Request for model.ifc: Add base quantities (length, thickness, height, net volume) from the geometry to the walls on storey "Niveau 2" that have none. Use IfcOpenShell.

First a look at what the model holds.

```python
import ifcopenshell
import ifcopenshell.util.element
import ifcopenshell.util.unit

model = ifcopenshell.open("model.ifc")
print(model.schema)
for unit_type in ("LENGTHUNIT", "AREAUNIT", "VOLUMEUNIT"):
    print(unit_type, ifcopenshell.util.unit.calculate_unit_scale(model, unit_type))
storey = next(s for s in model.by_type("IfcBuildingStorey") if s.Name == "Niveau 2")
walls = [e for e in ifcopenshell.util.element.get_decomposition(storey) if e.is_a("IfcWall")]
for e in sorted(walls, key=lambda e: e.id()):
    print(e.id(), e.is_a(), e.Name, list(ifcopenshell.util.element.get_psets(e, qtos_only=True)), sep=" | ")
```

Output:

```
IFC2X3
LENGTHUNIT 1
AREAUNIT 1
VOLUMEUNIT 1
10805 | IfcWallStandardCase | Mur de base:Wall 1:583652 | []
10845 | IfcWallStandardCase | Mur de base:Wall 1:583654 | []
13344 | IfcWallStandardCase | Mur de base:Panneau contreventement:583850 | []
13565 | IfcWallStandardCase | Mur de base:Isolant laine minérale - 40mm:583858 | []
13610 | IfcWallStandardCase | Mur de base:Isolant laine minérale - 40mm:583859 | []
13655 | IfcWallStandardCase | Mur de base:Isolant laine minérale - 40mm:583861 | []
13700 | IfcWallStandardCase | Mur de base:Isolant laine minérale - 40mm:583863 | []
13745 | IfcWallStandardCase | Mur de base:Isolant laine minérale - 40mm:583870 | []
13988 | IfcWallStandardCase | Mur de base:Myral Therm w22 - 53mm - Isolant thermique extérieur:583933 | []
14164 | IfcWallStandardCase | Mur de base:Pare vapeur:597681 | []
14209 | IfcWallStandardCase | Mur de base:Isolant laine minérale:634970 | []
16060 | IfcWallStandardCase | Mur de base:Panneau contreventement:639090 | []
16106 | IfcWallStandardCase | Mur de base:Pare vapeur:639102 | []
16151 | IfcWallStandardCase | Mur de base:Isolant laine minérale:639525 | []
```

```python
import ifcopenshell
import ifcopenshell.api.pset
import ifcopenshell.geom
import ifcopenshell.util.element
import ifcopenshell.util.shape
import ifcopenshell.util.unit

model = ifcopenshell.open("model.ifc")
unit_scale = ifcopenshell.util.unit.calculate_unit_scale(model)
volume_scale = ifcopenshell.util.unit.calculate_unit_scale(model, "VOLUMEUNIT")
settings = ifcopenshell.geom.settings()

storey = next(s for s in model.by_type("IfcBuildingStorey") if s.Name == "Niveau 2")
walls = [e for e in ifcopenshell.util.element.get_decomposition(storey) if e.is_a("IfcWall")]

for e in sorted(walls, key=lambda e: e.id()):
    if ifcopenshell.util.element.get_psets(e, qtos_only=True, should_inherit=False):
        continue
    # Geometry comes back in metres, in the element's own axes.
    shape = ifcopenshell.geom.create_shape(settings, e)
    values = {
        "Length": ifcopenshell.util.shape.get_x(shape.geometry) / unit_scale,
        "Width": ifcopenshell.util.shape.get_y(shape.geometry) / unit_scale,
        "Height": ifcopenshell.util.shape.get_z(shape.geometry) / unit_scale,
        "NetVolume": ifcopenshell.util.shape.get_volume(shape.geometry) / volume_scale,
    }
    qto = ifcopenshell.api.pset.add_qto(model, product=e, name="BaseQuantities")
    ifcopenshell.api.pset.edit_qto(model, qto=qto, properties=values)
    print(e.id(), {k: round(v, 3) for k, v in values.items()})

model.write("model-out.ifc")
```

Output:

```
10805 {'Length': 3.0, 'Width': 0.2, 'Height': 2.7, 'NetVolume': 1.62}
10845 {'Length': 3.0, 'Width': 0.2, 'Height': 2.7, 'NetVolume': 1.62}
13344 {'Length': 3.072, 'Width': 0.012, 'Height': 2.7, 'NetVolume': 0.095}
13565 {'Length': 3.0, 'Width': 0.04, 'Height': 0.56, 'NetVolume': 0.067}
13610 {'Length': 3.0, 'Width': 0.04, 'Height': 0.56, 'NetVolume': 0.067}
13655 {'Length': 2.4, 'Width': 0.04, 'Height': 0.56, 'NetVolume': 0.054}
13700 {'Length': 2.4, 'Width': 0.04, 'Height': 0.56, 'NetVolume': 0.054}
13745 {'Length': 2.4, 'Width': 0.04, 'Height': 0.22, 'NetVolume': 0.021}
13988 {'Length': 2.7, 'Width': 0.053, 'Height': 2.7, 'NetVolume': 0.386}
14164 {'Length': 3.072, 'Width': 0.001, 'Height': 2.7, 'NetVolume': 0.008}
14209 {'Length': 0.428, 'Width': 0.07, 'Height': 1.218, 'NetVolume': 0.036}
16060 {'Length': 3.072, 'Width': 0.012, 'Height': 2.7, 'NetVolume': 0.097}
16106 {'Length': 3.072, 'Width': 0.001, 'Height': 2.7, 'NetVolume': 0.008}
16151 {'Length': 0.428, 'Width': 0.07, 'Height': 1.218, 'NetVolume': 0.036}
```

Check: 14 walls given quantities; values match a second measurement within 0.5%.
